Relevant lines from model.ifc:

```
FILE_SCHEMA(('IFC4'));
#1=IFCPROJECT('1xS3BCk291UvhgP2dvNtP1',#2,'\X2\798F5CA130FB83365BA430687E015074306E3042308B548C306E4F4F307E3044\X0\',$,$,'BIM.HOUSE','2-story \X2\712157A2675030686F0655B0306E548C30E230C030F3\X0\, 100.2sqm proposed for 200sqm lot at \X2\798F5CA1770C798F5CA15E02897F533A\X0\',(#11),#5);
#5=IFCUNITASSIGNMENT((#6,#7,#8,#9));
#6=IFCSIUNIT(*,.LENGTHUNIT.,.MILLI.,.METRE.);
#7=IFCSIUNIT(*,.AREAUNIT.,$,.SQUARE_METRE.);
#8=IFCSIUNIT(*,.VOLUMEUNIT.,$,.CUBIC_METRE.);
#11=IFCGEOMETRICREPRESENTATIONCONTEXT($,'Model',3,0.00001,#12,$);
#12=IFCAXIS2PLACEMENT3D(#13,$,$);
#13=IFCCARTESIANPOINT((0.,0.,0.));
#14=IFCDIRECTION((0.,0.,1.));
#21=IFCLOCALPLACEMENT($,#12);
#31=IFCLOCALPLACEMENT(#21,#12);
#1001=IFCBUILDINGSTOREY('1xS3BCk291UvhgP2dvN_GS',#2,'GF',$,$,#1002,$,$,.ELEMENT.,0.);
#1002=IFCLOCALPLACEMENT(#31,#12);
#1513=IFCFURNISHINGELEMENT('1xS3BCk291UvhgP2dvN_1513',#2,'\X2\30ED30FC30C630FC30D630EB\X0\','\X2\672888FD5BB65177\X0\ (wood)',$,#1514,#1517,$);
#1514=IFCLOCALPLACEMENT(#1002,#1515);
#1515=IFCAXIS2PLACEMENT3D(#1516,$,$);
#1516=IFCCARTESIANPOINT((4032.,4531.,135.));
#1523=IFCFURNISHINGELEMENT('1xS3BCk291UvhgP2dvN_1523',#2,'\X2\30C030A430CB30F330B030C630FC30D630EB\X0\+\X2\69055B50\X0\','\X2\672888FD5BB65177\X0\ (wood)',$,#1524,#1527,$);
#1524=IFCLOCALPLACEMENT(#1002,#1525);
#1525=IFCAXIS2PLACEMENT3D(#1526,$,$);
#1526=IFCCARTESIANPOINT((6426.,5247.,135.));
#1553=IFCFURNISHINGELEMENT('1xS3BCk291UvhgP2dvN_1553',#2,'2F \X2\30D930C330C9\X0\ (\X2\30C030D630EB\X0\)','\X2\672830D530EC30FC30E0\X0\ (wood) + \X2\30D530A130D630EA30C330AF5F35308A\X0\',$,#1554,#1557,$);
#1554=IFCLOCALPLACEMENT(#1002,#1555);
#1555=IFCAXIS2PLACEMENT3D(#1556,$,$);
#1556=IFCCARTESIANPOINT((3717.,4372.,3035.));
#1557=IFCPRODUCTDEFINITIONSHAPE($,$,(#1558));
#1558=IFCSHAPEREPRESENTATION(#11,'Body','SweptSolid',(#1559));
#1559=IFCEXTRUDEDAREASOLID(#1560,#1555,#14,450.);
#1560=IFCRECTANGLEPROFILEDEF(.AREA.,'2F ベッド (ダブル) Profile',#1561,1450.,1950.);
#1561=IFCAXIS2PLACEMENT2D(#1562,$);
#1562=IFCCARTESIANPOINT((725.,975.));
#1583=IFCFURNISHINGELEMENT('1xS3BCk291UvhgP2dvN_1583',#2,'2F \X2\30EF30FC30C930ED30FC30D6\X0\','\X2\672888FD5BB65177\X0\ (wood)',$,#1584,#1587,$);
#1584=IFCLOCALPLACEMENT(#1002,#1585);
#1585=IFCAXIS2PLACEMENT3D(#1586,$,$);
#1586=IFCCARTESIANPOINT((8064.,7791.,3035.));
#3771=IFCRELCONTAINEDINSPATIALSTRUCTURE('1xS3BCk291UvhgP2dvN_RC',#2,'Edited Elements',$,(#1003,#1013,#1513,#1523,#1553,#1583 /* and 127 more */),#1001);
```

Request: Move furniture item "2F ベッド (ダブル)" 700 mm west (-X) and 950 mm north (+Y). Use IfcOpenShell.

```python
import ifcopenshell
import ifcopenshell.api.geometry
import ifcopenshell.util.placement
import ifcopenshell.util.unit

model = ifcopenshell.open("model.ifc")
unit_scale = ifcopenshell.util.unit.calculate_unit_scale(model)

item = model.by_id(1553)
matrix = ifcopenshell.util.placement.get_local_placement(item.ObjectPlacement)
matrix[0, 3] -= 0.7 / unit_scale
matrix[1, 3] += 0.95 / unit_scale
ifcopenshell.api.geometry.edit_object_placement(model, product=item, matrix=matrix, is_si=False)

print(ifcopenshell.util.placement.get_local_placement(item.ObjectPlacement).round(3) + 0.0)

model.write("model_v2.ifc")
```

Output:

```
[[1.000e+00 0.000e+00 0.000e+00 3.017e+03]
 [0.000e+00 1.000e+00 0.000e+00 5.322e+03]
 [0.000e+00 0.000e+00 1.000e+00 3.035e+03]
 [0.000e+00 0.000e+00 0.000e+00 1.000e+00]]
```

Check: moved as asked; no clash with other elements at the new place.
